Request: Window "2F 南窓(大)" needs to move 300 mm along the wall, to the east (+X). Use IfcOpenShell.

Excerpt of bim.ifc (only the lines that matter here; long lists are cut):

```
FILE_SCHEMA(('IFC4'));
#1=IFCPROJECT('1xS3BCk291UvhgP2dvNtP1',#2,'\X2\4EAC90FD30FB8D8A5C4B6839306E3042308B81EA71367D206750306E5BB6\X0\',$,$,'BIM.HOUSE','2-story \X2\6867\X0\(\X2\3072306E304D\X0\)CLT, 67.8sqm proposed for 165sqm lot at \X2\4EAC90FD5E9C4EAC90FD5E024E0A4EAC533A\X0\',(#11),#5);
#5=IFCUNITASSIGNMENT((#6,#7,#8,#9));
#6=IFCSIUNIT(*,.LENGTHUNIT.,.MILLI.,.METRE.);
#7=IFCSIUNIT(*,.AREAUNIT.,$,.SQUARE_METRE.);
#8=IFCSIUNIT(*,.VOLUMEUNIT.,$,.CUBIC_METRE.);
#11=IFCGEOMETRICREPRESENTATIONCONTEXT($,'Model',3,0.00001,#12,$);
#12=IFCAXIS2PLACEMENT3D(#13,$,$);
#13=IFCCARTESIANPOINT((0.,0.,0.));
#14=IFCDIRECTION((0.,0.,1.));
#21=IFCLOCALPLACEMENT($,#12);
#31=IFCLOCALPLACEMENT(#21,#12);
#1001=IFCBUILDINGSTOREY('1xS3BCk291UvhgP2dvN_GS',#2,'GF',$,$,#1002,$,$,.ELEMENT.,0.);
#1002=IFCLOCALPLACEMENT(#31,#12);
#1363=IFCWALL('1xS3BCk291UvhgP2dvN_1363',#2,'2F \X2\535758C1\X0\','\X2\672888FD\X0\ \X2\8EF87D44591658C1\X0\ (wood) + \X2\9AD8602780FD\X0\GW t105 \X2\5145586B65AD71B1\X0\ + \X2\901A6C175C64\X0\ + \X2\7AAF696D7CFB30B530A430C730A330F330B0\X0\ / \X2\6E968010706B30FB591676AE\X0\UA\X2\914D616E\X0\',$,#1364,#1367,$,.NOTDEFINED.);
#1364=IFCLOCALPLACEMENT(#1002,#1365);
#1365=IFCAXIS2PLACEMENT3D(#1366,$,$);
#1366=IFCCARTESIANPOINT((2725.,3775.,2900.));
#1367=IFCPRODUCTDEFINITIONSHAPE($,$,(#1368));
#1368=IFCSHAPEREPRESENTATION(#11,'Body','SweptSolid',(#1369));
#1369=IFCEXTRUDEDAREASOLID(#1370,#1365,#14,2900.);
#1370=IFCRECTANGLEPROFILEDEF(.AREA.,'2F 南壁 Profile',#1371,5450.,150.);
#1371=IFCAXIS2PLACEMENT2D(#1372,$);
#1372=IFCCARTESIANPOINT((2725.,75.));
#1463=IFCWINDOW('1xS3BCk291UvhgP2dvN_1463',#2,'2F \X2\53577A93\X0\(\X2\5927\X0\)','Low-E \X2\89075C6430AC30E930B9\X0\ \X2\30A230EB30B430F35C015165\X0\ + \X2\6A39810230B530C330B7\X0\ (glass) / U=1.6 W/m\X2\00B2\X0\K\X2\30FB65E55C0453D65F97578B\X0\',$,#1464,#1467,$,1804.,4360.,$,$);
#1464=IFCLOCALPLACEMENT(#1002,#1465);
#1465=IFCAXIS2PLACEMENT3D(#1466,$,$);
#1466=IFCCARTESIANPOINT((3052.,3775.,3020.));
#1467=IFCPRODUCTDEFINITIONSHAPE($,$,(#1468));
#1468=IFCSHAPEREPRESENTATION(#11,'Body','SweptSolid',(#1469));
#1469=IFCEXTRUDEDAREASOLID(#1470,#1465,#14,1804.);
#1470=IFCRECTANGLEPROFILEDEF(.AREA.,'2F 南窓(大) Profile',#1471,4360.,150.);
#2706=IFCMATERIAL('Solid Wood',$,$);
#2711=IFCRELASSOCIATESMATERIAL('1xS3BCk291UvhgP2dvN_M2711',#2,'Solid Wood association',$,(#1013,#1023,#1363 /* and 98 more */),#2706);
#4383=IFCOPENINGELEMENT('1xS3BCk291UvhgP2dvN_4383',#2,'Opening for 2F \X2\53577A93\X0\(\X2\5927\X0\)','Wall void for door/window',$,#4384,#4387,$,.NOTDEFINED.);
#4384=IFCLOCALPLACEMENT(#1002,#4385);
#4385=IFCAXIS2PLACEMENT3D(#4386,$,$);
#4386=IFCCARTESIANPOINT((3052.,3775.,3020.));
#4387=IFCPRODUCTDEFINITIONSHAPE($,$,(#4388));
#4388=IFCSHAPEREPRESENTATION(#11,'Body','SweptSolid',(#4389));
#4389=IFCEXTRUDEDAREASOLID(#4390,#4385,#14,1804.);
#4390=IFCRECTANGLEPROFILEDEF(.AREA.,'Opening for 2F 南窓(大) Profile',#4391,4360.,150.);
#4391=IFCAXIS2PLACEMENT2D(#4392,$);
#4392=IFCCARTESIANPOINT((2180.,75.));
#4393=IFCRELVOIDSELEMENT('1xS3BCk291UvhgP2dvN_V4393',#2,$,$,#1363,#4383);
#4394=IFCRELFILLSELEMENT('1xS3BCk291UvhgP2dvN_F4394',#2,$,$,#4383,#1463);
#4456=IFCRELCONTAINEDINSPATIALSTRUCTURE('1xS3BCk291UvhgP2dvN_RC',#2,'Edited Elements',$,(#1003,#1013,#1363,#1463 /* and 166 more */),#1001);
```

```python
import ifcopenshell
import ifcopenshell.api.geometry
import ifcopenshell.util.placement

model = ifcopenshell.open("bim.ifc")

window = model.by_id(1463)
opening = window.FillsVoids[0].RelatingOpeningElement
wall = opening.VoidsElements[0].RelatingBuildingElement

wall_matrix = ifcopenshell.util.placement.get_local_placement(wall.ObjectPlacement)
shift = wall_matrix[:3, 0] * 300.0
before = ifcopenshell.util.placement.get_local_placement(window.ObjectPlacement)[:3, 3].copy()

# The window is not placed relative to its opening, so move both.
for product in (opening, window):
    matrix = ifcopenshell.util.placement.get_local_placement(product.ObjectPlacement)
    matrix[:3, 3] += shift
    ifcopenshell.api.geometry.edit_object_placement(model, product=product, matrix=matrix, is_si=False)

after = ifcopenshell.util.placement.get_local_placement(window.ObjectPlacement)[:3, 3]
print("window moved by", (after - before).round(3) + 0.0)

model.write("bim_rev.ifc")
```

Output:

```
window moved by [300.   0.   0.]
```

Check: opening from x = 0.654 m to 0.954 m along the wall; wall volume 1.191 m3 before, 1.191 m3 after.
